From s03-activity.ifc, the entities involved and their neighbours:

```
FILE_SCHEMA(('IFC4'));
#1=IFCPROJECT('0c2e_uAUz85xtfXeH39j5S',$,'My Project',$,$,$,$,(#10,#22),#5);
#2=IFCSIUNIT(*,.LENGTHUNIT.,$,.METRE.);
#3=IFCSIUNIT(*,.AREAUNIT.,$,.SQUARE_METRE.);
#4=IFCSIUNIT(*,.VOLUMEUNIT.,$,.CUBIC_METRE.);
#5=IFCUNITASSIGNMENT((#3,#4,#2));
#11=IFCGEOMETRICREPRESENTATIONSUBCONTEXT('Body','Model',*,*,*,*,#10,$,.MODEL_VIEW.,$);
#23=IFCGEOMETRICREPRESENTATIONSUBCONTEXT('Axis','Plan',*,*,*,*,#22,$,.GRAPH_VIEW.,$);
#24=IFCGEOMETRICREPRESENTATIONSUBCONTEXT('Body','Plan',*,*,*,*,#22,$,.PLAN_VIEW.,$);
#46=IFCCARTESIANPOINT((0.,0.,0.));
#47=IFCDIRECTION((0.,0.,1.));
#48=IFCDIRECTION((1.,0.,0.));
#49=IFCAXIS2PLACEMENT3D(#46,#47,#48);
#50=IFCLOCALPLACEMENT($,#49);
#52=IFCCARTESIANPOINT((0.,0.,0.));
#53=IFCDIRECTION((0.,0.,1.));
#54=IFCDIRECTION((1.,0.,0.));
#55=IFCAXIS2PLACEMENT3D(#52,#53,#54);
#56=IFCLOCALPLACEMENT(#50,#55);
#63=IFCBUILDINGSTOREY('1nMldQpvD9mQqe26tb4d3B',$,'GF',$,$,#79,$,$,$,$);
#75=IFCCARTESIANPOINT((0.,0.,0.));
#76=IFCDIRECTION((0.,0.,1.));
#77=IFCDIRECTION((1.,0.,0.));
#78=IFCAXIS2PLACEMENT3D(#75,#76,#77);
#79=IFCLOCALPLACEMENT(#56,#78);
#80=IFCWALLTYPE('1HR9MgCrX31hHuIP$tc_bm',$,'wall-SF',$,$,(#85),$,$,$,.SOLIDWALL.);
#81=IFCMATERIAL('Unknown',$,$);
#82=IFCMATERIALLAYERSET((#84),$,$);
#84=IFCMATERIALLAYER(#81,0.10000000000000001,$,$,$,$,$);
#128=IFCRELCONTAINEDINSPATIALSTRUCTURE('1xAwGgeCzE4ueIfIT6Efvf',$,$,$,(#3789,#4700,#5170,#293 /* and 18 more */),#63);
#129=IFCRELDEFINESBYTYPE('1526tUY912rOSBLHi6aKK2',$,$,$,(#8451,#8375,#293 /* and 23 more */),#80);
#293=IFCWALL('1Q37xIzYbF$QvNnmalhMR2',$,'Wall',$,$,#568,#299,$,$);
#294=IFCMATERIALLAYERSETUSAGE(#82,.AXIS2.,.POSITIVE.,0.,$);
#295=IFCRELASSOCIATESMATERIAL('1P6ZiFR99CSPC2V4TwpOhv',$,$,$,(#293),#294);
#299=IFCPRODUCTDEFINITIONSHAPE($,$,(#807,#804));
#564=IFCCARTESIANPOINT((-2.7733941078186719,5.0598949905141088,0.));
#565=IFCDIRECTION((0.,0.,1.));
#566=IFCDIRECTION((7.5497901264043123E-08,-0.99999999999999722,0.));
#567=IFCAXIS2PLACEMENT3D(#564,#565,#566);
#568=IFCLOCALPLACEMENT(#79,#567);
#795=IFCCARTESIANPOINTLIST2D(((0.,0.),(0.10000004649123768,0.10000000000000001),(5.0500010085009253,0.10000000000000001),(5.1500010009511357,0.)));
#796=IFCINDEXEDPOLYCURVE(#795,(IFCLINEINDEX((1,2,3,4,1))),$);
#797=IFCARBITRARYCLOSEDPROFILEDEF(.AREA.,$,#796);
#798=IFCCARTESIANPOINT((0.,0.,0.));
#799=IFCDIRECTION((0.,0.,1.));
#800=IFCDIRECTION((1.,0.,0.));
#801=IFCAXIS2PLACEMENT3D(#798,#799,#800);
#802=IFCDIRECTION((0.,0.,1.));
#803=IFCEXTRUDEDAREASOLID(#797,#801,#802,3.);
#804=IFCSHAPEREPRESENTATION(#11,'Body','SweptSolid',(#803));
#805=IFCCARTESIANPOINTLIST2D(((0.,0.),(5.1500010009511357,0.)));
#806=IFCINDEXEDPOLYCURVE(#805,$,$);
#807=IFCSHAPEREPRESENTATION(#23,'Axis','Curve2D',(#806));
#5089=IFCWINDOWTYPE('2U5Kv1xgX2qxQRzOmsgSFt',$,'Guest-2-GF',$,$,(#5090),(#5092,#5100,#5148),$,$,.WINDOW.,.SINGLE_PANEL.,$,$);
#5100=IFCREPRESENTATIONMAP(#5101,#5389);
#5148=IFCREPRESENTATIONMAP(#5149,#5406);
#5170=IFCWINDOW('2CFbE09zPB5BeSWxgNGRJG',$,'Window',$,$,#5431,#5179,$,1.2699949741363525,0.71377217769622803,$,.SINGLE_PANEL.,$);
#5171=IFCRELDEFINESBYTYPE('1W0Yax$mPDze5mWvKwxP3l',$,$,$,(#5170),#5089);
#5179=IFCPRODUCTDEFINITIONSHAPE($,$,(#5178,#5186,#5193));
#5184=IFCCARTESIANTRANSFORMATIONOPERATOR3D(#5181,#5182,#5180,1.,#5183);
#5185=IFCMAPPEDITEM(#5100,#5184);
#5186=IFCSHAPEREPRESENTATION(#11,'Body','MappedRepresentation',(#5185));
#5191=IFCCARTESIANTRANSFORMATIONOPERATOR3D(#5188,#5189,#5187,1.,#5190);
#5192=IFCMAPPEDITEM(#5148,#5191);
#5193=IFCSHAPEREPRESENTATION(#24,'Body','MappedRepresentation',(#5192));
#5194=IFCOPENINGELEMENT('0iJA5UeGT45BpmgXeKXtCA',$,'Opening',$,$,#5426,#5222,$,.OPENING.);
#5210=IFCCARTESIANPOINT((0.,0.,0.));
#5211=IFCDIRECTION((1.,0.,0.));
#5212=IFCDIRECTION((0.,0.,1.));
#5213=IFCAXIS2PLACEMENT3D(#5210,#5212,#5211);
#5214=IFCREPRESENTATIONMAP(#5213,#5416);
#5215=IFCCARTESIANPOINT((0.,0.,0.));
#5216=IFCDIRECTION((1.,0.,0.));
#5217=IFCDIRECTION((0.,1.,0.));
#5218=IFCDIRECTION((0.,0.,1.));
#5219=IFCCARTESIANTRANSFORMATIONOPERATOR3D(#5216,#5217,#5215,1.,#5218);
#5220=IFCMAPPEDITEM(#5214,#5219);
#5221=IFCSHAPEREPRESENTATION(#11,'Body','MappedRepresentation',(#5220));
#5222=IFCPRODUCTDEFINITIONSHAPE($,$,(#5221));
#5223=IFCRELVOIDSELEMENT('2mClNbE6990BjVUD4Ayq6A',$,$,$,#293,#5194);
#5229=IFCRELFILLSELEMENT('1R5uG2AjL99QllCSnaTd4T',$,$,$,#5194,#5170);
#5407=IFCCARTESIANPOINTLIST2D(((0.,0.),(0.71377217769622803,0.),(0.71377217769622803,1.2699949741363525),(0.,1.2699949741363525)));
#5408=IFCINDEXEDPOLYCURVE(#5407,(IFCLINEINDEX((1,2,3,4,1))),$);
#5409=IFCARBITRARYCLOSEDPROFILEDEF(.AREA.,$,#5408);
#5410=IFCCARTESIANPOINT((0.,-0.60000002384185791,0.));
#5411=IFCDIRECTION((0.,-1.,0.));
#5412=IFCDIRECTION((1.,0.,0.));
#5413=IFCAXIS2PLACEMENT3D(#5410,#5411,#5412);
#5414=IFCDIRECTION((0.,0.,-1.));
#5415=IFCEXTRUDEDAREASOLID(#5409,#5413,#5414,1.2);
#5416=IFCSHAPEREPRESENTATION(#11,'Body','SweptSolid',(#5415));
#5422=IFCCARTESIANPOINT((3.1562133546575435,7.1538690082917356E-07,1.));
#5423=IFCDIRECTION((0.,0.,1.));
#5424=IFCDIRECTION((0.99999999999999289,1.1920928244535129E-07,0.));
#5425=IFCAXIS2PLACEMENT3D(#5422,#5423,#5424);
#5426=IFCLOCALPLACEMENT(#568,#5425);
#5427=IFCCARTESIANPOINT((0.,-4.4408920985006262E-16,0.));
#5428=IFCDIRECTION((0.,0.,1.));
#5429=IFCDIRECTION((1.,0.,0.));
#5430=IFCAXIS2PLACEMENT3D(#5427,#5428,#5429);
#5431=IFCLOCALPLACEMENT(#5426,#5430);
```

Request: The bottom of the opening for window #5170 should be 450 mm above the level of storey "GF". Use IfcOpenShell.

```python
import numpy as np
import ifcopenshell
import ifcopenshell.api.geometry
import ifcopenshell.geom
import ifcopenshell.util.element
import ifcopenshell.util.placement
import ifcopenshell.util.shape
import ifcopenshell.util.unit

model = ifcopenshell.open("s03-activity.ifc")
unit_scale = ifcopenshell.util.unit.calculate_unit_scale(model)

window = model.by_id(5170)
opening = window.FillsVoids[0].RelatingOpeningElement
storey = ifcopenshell.util.element.get_container(window, ifc_class="IfcBuildingStorey")
level = ifcopenshell.util.placement.get_local_placement(storey.ObjectPlacement)[2, 3]

# The opening's origin need not be at the sill, so measure its lowest point.
shape = ifcopenshell.geom.create_shape(ifcopenshell.geom.settings(), opening)
bottom = ifcopenshell.util.shape.get_shape_bottom_elevation(shape, shape.geometry) / unit_scale
dz = level + 0.45 / unit_scale - bottom

shift = np.array([0.0, 0.0, dz])
# The window is placed relative to its opening, so it follows when the opening moves.
matrix = ifcopenshell.util.placement.get_local_placement(opening.ObjectPlacement)
matrix[:3, 3] += shift
ifcopenshell.api.geometry.edit_object_placement(
    model, product=opening, matrix=matrix, is_si=False, should_transform_children=True
)

print(f"moved by {dz * unit_scale:+.3f} m")

model.write("s03-activity_edited.ifc")
```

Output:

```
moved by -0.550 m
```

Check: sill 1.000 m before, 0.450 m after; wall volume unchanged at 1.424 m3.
